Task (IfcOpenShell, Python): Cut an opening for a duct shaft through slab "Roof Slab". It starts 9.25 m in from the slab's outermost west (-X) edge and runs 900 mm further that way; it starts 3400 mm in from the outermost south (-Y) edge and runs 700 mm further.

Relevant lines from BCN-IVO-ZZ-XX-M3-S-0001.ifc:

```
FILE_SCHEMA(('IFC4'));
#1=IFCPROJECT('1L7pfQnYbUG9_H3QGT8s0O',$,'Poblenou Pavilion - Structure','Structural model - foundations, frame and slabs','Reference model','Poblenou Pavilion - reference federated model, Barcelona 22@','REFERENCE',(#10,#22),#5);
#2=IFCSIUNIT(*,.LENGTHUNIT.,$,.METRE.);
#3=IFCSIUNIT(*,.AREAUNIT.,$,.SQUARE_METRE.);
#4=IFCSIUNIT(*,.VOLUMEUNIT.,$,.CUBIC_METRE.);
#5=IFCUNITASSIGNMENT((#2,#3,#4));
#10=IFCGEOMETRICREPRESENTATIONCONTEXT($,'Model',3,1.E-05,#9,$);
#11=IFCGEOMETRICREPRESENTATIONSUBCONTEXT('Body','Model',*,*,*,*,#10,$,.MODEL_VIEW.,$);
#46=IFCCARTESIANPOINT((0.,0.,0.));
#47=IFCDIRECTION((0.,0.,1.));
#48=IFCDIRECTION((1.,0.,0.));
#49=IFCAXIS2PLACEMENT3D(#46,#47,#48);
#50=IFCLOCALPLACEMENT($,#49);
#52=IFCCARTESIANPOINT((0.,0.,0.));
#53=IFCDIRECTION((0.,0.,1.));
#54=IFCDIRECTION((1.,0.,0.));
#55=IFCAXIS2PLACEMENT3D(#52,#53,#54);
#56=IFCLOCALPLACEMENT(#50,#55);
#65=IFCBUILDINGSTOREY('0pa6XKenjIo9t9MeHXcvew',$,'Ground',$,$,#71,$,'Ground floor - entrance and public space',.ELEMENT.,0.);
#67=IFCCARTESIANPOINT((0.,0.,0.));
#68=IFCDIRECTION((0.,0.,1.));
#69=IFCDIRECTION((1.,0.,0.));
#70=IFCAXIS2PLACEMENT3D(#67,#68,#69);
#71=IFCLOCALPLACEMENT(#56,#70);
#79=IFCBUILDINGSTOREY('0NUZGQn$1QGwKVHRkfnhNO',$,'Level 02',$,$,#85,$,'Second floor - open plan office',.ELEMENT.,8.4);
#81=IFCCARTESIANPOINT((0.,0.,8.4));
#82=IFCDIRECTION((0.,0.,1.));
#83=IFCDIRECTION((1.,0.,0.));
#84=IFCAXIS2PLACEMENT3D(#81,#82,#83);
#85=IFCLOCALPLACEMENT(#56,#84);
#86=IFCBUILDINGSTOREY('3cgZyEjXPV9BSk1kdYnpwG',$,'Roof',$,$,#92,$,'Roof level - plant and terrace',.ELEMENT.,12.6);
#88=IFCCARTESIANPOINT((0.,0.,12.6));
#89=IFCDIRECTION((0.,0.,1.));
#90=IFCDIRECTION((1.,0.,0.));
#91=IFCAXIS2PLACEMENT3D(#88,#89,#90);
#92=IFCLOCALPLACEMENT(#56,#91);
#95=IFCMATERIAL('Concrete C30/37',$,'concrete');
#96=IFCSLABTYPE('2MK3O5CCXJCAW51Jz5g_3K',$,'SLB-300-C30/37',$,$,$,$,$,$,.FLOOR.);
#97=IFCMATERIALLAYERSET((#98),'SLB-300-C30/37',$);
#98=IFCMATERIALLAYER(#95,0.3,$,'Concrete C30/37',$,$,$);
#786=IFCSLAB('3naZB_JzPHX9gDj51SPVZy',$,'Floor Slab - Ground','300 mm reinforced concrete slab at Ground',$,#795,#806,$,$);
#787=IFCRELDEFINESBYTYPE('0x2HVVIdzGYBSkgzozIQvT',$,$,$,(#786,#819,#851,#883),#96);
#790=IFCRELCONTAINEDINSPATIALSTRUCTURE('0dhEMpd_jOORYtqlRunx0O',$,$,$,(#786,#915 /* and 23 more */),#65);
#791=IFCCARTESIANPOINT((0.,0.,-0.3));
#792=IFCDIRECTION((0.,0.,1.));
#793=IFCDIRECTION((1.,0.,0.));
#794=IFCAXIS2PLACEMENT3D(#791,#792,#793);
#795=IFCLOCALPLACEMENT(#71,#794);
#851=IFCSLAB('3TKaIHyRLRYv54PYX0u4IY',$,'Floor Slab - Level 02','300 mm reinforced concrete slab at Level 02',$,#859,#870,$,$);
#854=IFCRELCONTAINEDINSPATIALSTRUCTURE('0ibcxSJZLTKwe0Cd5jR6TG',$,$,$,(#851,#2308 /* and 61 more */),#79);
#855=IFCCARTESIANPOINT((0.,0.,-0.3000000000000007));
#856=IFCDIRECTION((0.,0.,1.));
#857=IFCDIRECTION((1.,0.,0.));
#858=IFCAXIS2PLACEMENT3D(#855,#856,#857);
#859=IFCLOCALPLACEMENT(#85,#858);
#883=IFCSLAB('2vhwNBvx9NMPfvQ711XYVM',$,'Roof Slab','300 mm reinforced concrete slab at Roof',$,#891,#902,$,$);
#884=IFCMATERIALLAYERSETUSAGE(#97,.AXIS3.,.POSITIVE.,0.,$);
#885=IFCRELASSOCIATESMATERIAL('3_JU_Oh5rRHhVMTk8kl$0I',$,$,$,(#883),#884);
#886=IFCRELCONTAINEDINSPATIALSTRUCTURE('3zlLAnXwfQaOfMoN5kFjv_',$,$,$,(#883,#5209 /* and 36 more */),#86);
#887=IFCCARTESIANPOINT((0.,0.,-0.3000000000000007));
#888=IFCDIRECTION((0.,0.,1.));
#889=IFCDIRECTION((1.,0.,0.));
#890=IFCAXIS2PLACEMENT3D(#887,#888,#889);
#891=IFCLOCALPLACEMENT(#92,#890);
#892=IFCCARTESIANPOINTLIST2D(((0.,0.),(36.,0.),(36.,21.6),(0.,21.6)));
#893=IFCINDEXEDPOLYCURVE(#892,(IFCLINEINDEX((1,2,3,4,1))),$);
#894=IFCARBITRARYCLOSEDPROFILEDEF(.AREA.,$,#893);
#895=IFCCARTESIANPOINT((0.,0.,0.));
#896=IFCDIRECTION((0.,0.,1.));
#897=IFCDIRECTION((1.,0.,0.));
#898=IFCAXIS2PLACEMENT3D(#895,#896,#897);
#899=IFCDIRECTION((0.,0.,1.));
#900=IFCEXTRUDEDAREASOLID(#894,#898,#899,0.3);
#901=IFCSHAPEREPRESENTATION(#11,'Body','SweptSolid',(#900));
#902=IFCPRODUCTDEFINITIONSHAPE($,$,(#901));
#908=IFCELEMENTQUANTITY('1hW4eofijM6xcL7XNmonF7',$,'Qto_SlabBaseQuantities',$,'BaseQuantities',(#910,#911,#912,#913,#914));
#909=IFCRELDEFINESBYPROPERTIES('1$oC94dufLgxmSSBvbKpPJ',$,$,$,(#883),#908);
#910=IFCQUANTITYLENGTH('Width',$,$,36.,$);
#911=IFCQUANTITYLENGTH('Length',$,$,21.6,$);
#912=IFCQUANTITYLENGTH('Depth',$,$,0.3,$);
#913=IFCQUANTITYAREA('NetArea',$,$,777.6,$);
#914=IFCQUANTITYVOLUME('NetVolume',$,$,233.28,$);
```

```python
import numpy as np
import ifcopenshell
import ifcopenshell.api.feature
import ifcopenshell.api.geometry
import ifcopenshell.api.pset
import ifcopenshell.api.root
import ifcopenshell.geom
import ifcopenshell.util.element
import ifcopenshell.util.placement
import ifcopenshell.util.representation
import ifcopenshell.util.shape
import ifcopenshell.util.unit

model = ifcopenshell.open("BCN-IVO-ZZ-XX-M3-S-0001.ifc")
unit_scale = ifcopenshell.util.unit.calculate_unit_scale(model)
area_scale = ifcopenshell.util.unit.calculate_unit_scale(model, "AREAUNIT")
volume_scale = ifcopenshell.util.unit.calculate_unit_scale(model, "VOLUMEUNIT")
settings = ifcopenshell.geom.settings()


def volume(element):
    """Net volume in cubic metres, openings subtracted."""
    shape = ifcopenshell.geom.create_shape(settings, element)
    return ifcopenshell.util.shape.get_volume(shape.geometry)


slab = model.by_guid("2vhwNBvx9NMPfvQ711XYVM")
before = volume(slab)

# Extent in the slab's own axes, in metres. The edges named are its -X and -Y sides.
slab_shape = ifcopenshell.geom.create_shape(settings, slab)
vertices = ifcopenshell.util.shape.get_vertices(slab_shape.geometry)
x_min, y_min, bottom = vertices.min(axis=0)
top = vertices[:, 2].max()

opening = ifcopenshell.api.root.create_entity(model, ifc_class="IfcOpeningElement", name="Duct shaft opening", predefined_type="OPENING")
context = ifcopenshell.util.representation.get_context(model, "Model", "Body", "MODEL_VIEW")
width, depth = 0.9, 0.7
outline = [(0.0, 0.0), (width, 0.0), (width, depth), (0.0, depth), (0.0, 0.0)]
# Overshoot both faces by 50 mm so the cut is clean.
shape = ifcopenshell.api.geometry.add_slab_representation(
    model, context=context, depth=top - bottom + 0.1, polyline=outline
)
ifcopenshell.api.geometry.assign_representation(model, product=opening, representation=shape)

matrix = ifcopenshell.util.placement.get_local_placement(slab.ObjectPlacement)
matrix[:, 3] = matrix @ np.append(np.array([x_min + 9.25, y_min + 3.4, bottom - 0.05]) / unit_scale, 1.0)
ifcopenshell.api.geometry.edit_object_placement(model, product=opening, matrix=matrix, is_si=False)
ifcopenshell.api.feature.add_feature(model, feature=opening, element=slab)

after = volume(slab)

# Update the slab's stored quantities.
qto = model.by_id(ifcopenshell.util.element.get_pset(slab, "Qto_SlabBaseQuantities", should_inherit=False)["id"])
ifcopenshell.api.pset.edit_qto(model, qto=qto, properties={
    "NetArea": after / (top - bottom) / area_scale,
    "NetVolume": after / volume_scale,
})

print(f"slab volume {before:.3f} -> {after:.3f} m3")

model.write("BCN-IVO-ZZ-XX-M3-S-0001_edited.ifc")
```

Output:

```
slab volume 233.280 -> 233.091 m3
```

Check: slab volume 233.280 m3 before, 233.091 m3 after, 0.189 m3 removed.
